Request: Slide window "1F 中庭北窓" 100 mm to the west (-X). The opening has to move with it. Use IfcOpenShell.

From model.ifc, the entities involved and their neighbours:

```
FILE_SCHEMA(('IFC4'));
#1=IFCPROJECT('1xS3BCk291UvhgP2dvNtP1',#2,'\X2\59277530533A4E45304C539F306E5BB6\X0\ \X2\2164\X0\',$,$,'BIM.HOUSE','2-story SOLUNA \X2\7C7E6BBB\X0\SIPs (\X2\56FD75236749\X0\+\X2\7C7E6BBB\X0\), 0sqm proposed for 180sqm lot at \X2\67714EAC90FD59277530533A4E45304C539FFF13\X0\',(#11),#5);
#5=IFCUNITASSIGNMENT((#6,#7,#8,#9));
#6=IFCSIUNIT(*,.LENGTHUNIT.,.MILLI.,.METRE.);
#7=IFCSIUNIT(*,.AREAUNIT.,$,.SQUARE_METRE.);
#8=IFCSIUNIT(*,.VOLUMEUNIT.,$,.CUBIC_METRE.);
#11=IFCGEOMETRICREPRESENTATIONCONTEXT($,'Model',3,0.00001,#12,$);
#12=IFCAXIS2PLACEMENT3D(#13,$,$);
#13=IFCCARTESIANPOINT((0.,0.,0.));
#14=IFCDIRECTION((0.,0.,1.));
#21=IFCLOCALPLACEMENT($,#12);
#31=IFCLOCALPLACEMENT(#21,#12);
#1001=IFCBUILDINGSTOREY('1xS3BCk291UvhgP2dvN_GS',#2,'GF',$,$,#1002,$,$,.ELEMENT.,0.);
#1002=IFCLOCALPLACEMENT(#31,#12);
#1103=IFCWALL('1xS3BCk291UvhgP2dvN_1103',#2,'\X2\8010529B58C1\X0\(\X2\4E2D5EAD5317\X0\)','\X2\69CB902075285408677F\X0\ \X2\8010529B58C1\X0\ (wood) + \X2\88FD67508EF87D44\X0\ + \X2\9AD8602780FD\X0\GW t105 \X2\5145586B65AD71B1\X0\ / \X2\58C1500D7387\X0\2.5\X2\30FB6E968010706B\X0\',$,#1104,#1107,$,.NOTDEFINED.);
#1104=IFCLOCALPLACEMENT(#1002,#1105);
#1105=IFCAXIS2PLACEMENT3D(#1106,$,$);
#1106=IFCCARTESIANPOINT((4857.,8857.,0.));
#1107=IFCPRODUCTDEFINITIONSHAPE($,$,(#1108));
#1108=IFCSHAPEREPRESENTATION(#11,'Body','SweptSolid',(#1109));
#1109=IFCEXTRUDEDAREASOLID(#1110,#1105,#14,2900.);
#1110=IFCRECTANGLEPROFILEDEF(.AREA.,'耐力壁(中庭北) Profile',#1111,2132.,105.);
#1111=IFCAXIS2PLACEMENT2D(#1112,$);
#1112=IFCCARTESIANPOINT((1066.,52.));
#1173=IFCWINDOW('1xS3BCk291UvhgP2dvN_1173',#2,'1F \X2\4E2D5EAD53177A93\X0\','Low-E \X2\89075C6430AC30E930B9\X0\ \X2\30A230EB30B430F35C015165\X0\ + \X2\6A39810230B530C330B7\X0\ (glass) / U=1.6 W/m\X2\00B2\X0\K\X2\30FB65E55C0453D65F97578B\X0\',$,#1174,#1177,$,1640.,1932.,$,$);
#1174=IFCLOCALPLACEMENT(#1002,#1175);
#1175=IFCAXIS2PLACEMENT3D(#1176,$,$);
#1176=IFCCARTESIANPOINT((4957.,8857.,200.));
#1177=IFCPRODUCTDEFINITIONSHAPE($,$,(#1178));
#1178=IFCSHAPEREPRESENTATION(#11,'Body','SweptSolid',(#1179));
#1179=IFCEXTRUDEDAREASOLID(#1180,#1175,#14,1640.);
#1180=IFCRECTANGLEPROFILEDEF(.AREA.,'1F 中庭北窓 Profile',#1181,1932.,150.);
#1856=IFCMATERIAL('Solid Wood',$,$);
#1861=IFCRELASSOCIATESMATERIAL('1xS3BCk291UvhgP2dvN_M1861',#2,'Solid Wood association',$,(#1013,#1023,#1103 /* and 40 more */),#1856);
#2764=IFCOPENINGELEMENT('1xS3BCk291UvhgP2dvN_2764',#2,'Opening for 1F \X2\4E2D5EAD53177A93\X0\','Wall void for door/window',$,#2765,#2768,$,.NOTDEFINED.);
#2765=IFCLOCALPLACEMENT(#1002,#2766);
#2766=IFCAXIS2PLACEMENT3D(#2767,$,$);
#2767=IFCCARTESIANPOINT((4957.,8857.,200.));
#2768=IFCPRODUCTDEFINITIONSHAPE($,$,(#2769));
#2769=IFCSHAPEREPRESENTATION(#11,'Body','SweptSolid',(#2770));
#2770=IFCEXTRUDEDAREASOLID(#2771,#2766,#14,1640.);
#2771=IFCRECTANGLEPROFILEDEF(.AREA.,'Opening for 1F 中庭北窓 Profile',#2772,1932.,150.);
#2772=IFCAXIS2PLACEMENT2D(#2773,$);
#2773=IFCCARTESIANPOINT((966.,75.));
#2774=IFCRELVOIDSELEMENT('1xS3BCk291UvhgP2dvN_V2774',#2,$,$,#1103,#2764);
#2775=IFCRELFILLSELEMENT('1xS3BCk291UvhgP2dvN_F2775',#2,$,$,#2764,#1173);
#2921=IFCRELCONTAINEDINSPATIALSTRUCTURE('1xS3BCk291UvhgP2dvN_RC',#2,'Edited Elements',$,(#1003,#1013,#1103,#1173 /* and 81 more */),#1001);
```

```python
import ifcopenshell
import ifcopenshell.api.geometry
import ifcopenshell.util.placement
import ifcopenshell.util.unit

model = ifcopenshell.open("model.ifc")
unit_scale = ifcopenshell.util.unit.calculate_unit_scale(model)

window = model.by_guid("1xS3BCk291UvhgP2dvN_1173")
opening = window.FillsVoids[0].RelatingOpeningElement
wall = opening.VoidsElements[0].RelatingBuildingElement

wall_matrix = ifcopenshell.util.placement.get_local_placement(wall.ObjectPlacement)
shift = wall_matrix[:3, 0] * -0.1 / unit_scale
before = ifcopenshell.util.placement.get_local_placement(window.ObjectPlacement)[:3, 3].copy()

# The window is not placed relative to its opening, so move both.
for product in (opening, window):
    matrix = ifcopenshell.util.placement.get_local_placement(product.ObjectPlacement)
    matrix[:3, 3] += shift
    ifcopenshell.api.geometry.edit_object_placement(model, product=product, matrix=matrix, is_si=False)

after = ifcopenshell.util.placement.get_local_placement(window.ObjectPlacement)[:3, 3]
print("window moved by", (after - before).round(3) + 0.0)

model.write("model_updated.ifc")
```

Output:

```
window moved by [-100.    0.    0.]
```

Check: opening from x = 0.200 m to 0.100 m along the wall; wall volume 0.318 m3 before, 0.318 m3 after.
